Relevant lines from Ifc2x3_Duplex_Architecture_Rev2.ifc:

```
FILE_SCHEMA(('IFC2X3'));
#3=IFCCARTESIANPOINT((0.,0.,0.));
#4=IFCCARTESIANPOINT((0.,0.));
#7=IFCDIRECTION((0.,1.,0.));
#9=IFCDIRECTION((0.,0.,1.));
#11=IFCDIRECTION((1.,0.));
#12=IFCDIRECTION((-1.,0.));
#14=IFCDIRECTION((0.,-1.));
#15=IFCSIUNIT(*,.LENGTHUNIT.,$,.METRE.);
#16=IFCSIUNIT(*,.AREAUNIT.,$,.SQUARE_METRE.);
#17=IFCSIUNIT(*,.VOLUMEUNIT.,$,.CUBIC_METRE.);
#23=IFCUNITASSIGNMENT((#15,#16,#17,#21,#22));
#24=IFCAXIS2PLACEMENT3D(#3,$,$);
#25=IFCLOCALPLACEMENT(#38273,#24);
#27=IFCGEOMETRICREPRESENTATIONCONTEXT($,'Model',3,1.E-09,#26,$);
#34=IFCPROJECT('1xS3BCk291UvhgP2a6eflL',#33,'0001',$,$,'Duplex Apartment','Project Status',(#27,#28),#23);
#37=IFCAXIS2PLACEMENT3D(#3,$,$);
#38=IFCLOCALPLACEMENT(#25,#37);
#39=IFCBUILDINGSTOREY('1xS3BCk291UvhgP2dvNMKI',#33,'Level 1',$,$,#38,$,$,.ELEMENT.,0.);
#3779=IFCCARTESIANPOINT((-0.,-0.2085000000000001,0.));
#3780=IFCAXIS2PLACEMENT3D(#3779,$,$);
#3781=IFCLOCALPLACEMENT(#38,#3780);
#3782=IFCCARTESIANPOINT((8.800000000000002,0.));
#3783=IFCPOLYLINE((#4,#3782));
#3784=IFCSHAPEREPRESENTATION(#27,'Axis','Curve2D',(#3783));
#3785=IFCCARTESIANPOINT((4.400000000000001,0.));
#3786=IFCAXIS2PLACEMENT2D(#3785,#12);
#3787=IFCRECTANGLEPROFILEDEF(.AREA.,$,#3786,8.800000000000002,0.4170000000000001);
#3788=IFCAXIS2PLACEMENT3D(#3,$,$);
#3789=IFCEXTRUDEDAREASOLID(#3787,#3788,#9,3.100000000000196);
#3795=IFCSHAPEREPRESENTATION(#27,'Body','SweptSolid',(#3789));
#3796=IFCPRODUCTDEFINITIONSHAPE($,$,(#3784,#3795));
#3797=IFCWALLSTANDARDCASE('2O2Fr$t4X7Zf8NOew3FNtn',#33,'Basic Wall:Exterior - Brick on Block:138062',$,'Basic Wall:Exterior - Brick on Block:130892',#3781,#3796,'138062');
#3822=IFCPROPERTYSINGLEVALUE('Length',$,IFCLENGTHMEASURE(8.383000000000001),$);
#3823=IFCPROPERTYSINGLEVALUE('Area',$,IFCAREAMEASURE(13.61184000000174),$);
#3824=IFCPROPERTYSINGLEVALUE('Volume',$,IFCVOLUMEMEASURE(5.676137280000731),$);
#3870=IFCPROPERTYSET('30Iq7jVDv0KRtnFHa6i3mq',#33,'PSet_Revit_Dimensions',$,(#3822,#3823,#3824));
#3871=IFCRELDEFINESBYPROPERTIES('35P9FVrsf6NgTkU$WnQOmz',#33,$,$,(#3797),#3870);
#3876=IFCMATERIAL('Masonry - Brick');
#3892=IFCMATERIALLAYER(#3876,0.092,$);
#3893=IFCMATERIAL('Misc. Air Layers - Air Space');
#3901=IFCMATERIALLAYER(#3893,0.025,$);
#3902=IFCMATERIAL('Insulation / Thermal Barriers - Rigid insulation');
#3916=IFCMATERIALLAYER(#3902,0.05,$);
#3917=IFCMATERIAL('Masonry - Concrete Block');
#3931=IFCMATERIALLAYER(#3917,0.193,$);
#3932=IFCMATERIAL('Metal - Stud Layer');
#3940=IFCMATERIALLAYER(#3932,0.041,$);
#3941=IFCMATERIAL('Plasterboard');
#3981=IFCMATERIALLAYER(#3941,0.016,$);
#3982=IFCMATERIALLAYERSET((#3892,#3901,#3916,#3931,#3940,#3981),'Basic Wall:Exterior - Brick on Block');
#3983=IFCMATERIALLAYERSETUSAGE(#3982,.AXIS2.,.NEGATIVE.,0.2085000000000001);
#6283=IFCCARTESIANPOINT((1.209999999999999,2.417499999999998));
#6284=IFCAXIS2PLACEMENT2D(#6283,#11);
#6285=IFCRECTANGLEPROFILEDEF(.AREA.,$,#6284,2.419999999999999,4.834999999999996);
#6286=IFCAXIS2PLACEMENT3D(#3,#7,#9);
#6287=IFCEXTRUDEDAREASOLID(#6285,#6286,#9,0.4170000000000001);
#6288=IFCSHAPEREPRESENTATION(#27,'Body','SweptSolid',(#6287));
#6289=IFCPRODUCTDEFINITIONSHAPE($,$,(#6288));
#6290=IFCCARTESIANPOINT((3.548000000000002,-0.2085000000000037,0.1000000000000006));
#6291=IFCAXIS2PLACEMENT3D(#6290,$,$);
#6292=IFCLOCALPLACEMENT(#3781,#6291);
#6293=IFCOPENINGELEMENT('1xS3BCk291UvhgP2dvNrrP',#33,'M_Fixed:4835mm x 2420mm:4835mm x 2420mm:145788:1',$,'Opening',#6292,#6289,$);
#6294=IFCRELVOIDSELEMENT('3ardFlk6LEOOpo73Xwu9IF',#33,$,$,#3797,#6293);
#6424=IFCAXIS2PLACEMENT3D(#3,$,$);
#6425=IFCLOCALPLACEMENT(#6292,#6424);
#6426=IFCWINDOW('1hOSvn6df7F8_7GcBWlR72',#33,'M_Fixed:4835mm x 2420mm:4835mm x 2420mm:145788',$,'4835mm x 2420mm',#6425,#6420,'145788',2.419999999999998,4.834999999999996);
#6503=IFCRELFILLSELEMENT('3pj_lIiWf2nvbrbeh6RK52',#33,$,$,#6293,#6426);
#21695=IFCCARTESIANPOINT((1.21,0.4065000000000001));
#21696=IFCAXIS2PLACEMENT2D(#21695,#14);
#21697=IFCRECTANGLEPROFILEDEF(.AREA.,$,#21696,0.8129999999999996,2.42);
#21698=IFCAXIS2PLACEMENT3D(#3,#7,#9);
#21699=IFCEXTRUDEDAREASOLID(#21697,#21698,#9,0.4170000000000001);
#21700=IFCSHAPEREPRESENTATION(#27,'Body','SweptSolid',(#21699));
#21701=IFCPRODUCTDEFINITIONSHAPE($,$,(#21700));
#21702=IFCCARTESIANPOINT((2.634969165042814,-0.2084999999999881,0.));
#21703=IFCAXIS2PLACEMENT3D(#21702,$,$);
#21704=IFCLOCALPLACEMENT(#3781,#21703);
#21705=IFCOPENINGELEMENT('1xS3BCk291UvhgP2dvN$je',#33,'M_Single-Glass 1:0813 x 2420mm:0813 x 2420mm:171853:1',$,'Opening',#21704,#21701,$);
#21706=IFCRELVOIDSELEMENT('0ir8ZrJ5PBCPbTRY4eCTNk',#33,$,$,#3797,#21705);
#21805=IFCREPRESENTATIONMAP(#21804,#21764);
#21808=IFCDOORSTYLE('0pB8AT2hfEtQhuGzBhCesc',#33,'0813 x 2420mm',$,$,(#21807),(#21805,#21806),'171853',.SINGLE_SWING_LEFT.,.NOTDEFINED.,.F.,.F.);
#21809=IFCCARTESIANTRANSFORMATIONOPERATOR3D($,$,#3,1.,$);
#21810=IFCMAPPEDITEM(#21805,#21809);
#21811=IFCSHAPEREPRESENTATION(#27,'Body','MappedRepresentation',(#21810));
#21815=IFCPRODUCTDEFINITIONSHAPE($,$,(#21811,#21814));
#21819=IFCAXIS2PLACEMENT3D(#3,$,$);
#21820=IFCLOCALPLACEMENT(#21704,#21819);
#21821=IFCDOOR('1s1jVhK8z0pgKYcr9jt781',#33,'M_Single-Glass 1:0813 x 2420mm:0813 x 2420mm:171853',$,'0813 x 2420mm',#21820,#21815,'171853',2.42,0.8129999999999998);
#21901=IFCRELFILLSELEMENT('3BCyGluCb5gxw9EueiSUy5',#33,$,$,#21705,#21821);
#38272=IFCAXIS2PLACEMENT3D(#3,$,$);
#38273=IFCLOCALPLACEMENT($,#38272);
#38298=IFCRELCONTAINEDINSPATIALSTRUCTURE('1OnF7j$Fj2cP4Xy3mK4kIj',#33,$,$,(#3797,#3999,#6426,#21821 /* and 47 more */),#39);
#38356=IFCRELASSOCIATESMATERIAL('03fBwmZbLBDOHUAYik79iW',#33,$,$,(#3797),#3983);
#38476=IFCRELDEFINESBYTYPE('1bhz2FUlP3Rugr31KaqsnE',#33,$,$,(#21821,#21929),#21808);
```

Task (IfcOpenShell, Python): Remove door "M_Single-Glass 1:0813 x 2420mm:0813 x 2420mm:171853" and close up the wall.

```python
import ifcopenshell
import ifcopenshell.api.feature
import ifcopenshell.api.pset
import ifcopenshell.api.root
import ifcopenshell.geom
import ifcopenshell.util.element
import ifcopenshell.util.shape
import ifcopenshell.util.unit

model = ifcopenshell.open("Ifc2x3_Duplex_Architecture_Rev2.ifc")
area_scale = ifcopenshell.util.unit.calculate_unit_scale(model, "AREAUNIT")
volume_scale = ifcopenshell.util.unit.calculate_unit_scale(model, "VOLUMEUNIT")
settings = ifcopenshell.geom.settings()


def volume(element):
    """Net volume in cubic metres, openings subtracted."""
    shape = ifcopenshell.geom.create_shape(settings, element)
    return ifcopenshell.util.shape.get_volume(shape.geometry)


door = model.by_id(21821)
opening = door.FillsVoids[0].RelatingOpeningElement
wall = opening.VoidsElements[0].RelatingBuildingElement
before = volume(wall)

ifcopenshell.api.root.remove_product(model, product=door)
ifcopenshell.api.feature.remove_feature(model, feature=opening)

after = volume(wall)
thickness = 0.417  # wall thickness in metres

# Update the wall's stored quantities.
pset = model.by_id(ifcopenshell.util.element.get_pset(wall, "PSet_Revit_Dimensions", should_inherit=False)["id"])
ifcopenshell.api.pset.edit_pset(model, pset=pset, properties={
    "Area": model.create_entity("IfcAreaMeasure", after / thickness / area_scale),
    "Volume": model.create_entity("IfcVolumeMeasure", after / volume_scale),
})

print(f"wall volume {before:.3f} -> {after:.3f} m3")

model.write("Ifc2x3_Duplex_Architecture_Rev2_v2.ifc")
```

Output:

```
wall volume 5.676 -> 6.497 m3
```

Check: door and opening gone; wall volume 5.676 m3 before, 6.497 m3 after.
